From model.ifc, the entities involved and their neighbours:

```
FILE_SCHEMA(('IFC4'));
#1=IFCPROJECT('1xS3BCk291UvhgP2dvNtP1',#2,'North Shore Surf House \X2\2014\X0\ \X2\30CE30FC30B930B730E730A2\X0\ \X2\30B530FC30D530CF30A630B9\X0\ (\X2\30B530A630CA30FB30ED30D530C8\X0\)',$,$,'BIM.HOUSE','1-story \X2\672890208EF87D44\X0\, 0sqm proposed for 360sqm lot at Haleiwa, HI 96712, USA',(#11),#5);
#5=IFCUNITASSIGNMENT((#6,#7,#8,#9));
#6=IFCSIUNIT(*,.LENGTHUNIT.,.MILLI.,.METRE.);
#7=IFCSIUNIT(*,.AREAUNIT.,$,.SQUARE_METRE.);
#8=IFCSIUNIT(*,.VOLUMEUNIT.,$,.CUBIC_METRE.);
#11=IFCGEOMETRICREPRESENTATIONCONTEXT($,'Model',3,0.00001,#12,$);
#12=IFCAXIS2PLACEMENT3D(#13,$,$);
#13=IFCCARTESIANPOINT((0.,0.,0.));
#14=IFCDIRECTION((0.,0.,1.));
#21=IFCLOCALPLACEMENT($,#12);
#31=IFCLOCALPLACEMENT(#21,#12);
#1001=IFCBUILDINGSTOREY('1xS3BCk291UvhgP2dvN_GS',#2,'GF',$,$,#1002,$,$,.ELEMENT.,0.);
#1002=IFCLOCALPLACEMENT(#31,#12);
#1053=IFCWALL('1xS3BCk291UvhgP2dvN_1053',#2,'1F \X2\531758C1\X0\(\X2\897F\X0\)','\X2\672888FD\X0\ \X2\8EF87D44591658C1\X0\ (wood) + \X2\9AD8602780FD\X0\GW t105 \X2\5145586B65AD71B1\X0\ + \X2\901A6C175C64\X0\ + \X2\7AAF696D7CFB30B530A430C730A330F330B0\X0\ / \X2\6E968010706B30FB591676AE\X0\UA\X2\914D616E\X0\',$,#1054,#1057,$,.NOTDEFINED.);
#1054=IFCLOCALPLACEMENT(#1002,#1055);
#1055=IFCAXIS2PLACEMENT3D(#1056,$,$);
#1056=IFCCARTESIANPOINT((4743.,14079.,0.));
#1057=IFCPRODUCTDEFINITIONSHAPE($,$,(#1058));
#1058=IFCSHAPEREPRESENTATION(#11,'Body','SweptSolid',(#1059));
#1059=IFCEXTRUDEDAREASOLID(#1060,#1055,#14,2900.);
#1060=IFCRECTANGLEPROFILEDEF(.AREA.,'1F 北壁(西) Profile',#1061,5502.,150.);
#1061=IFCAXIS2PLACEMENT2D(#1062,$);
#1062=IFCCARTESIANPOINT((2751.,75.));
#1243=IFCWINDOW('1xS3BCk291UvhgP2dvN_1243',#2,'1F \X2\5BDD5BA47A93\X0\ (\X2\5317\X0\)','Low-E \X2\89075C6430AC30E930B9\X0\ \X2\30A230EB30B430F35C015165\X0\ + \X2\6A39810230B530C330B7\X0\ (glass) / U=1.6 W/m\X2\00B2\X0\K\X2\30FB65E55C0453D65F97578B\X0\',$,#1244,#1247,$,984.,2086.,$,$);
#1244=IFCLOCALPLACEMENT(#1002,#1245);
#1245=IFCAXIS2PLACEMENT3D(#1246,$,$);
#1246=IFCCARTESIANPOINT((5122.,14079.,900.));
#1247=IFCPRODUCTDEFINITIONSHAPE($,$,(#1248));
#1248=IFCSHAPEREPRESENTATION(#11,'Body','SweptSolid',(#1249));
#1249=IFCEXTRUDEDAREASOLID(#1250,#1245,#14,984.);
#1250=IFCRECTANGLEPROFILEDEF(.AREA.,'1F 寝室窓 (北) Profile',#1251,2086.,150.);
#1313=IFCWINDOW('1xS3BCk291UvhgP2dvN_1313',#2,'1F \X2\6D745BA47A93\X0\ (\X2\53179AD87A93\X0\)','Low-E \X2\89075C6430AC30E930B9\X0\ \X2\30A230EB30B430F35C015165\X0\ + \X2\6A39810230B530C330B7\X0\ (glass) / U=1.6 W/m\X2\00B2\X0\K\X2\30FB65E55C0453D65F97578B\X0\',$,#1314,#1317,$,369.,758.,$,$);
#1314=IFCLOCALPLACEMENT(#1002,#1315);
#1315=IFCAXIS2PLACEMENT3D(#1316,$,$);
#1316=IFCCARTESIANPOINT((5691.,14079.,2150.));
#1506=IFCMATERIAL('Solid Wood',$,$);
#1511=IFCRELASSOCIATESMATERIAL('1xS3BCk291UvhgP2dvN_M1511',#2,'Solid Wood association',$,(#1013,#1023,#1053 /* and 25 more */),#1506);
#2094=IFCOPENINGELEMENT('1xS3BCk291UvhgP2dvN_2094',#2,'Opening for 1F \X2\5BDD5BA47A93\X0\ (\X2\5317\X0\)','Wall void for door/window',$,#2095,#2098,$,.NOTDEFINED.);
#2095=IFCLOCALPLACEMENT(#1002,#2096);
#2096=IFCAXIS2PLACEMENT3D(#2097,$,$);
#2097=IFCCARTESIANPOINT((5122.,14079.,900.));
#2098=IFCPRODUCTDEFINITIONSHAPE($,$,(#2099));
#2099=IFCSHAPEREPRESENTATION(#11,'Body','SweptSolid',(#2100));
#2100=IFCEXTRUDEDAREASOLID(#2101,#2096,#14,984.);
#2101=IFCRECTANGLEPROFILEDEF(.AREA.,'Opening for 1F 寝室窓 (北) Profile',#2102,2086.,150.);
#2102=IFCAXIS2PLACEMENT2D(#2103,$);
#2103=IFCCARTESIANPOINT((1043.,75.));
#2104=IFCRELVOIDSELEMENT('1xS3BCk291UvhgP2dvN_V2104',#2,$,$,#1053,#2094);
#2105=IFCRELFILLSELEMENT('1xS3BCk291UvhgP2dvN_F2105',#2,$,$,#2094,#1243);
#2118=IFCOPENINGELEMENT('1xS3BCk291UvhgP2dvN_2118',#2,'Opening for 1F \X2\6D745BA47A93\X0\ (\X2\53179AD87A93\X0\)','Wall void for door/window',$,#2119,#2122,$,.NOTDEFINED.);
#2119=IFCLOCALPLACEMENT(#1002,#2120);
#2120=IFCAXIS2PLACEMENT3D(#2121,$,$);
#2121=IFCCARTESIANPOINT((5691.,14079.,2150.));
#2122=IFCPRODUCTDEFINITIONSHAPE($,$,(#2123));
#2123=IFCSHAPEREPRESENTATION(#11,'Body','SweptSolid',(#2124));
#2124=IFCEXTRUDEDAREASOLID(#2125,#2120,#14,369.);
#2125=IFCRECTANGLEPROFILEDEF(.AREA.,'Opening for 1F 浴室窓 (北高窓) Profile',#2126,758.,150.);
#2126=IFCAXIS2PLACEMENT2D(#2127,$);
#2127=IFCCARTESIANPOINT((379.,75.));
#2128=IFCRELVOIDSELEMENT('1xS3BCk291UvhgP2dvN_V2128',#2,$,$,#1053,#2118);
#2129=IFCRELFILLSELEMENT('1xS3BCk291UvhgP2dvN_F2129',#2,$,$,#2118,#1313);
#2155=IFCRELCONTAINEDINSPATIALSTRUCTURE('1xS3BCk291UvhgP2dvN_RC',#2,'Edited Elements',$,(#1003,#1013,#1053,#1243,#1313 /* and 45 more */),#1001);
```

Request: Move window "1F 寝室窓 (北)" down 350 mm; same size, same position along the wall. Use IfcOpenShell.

```python
import numpy as np
import ifcopenshell
import ifcopenshell.api.geometry
import ifcopenshell.util.placement
import ifcopenshell.util.unit

model = ifcopenshell.open("model.ifc")
unit_scale = ifcopenshell.util.unit.calculate_unit_scale(model)

window = model.by_guid("1xS3BCk291UvhgP2dvN_1243")
opening = window.FillsVoids[0].RelatingOpeningElement
dz = -0.35 / unit_scale

shift = np.array([0.0, 0.0, dz])
# The window is not placed relative to its opening, so move both.
for product in (opening, window):
    matrix = ifcopenshell.util.placement.get_local_placement(product.ObjectPlacement)
    matrix[:3, 3] += shift
    ifcopenshell.api.geometry.edit_object_placement(model, product=product, matrix=matrix, is_si=False)

print(f"moved by {dz * unit_scale:+.3f} m")

model.write("model_updated.ifc")
```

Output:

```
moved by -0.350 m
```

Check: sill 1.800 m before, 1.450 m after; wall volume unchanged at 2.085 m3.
